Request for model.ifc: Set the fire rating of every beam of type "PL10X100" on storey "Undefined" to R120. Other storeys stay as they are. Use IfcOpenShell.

First a look at what the model holds.

```python
import ifcopenshell
import ifcopenshell.util.element

model = ifcopenshell.open("model.ifc")
print(model.schema)
storey = next(s for s in model.by_type("IfcBuildingStorey") if s.Name == "Undefined")
beams = [e for e in ifcopenshell.util.element.get_decomposition(storey) if e.is_a("IfcBeam")]
seen = {}
for e in beams:
    element_type = ifcopenshell.util.element.get_type(e)
    key = (element_type.Name if element_type != e and element_type else None, ifcopenshell.util.element.get_pset(e, "Pset_BeamCommon", "FireRating"))
    seen[key] = seen.get(key, 0) + 1
for (name, value), count in sorted(seen.items(), key=str):
    print(count, "x", name, "|", value)
```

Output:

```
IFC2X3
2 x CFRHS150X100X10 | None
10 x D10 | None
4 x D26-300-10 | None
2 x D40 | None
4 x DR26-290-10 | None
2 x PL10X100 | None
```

```python
import ifcopenshell
import ifcopenshell.api.pset
import ifcopenshell.util.element

model = ifcopenshell.open("model.ifc")

storey = next(s for s in model.by_type("IfcBuildingStorey") if s.Name == "Undefined")
beams = [e for e in ifcopenshell.util.element.get_decomposition(storey) if e.is_a("IfcBeam")]

count = 0
for e in beams:
    element_type = ifcopenshell.util.element.get_type(e)
    if element_type in (None, e) or element_type.Name != "PL10X100":
        continue
    found = ifcopenshell.util.element.get_pset(e, "Pset_BeamCommon", should_inherit=False)
    if found:
        pset = model.by_id(found["id"])
        if len(ifcopenshell.util.element.get_elements_by_pset(pset)) > 1:
            pset = ifcopenshell.api.pset.unshare_pset(model, products=[e], pset=pset)[0]
    else:
        pset = ifcopenshell.api.pset.add_pset(model, product=e, name="Pset_BeamCommon")
    ifcopenshell.api.pset.edit_pset(model, pset=pset, properties={"FireRating": "R120"})
    count += 1

print(count, "beams updated")

model.write("model_edited.ifc")
```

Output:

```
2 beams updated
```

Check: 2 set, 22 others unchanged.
